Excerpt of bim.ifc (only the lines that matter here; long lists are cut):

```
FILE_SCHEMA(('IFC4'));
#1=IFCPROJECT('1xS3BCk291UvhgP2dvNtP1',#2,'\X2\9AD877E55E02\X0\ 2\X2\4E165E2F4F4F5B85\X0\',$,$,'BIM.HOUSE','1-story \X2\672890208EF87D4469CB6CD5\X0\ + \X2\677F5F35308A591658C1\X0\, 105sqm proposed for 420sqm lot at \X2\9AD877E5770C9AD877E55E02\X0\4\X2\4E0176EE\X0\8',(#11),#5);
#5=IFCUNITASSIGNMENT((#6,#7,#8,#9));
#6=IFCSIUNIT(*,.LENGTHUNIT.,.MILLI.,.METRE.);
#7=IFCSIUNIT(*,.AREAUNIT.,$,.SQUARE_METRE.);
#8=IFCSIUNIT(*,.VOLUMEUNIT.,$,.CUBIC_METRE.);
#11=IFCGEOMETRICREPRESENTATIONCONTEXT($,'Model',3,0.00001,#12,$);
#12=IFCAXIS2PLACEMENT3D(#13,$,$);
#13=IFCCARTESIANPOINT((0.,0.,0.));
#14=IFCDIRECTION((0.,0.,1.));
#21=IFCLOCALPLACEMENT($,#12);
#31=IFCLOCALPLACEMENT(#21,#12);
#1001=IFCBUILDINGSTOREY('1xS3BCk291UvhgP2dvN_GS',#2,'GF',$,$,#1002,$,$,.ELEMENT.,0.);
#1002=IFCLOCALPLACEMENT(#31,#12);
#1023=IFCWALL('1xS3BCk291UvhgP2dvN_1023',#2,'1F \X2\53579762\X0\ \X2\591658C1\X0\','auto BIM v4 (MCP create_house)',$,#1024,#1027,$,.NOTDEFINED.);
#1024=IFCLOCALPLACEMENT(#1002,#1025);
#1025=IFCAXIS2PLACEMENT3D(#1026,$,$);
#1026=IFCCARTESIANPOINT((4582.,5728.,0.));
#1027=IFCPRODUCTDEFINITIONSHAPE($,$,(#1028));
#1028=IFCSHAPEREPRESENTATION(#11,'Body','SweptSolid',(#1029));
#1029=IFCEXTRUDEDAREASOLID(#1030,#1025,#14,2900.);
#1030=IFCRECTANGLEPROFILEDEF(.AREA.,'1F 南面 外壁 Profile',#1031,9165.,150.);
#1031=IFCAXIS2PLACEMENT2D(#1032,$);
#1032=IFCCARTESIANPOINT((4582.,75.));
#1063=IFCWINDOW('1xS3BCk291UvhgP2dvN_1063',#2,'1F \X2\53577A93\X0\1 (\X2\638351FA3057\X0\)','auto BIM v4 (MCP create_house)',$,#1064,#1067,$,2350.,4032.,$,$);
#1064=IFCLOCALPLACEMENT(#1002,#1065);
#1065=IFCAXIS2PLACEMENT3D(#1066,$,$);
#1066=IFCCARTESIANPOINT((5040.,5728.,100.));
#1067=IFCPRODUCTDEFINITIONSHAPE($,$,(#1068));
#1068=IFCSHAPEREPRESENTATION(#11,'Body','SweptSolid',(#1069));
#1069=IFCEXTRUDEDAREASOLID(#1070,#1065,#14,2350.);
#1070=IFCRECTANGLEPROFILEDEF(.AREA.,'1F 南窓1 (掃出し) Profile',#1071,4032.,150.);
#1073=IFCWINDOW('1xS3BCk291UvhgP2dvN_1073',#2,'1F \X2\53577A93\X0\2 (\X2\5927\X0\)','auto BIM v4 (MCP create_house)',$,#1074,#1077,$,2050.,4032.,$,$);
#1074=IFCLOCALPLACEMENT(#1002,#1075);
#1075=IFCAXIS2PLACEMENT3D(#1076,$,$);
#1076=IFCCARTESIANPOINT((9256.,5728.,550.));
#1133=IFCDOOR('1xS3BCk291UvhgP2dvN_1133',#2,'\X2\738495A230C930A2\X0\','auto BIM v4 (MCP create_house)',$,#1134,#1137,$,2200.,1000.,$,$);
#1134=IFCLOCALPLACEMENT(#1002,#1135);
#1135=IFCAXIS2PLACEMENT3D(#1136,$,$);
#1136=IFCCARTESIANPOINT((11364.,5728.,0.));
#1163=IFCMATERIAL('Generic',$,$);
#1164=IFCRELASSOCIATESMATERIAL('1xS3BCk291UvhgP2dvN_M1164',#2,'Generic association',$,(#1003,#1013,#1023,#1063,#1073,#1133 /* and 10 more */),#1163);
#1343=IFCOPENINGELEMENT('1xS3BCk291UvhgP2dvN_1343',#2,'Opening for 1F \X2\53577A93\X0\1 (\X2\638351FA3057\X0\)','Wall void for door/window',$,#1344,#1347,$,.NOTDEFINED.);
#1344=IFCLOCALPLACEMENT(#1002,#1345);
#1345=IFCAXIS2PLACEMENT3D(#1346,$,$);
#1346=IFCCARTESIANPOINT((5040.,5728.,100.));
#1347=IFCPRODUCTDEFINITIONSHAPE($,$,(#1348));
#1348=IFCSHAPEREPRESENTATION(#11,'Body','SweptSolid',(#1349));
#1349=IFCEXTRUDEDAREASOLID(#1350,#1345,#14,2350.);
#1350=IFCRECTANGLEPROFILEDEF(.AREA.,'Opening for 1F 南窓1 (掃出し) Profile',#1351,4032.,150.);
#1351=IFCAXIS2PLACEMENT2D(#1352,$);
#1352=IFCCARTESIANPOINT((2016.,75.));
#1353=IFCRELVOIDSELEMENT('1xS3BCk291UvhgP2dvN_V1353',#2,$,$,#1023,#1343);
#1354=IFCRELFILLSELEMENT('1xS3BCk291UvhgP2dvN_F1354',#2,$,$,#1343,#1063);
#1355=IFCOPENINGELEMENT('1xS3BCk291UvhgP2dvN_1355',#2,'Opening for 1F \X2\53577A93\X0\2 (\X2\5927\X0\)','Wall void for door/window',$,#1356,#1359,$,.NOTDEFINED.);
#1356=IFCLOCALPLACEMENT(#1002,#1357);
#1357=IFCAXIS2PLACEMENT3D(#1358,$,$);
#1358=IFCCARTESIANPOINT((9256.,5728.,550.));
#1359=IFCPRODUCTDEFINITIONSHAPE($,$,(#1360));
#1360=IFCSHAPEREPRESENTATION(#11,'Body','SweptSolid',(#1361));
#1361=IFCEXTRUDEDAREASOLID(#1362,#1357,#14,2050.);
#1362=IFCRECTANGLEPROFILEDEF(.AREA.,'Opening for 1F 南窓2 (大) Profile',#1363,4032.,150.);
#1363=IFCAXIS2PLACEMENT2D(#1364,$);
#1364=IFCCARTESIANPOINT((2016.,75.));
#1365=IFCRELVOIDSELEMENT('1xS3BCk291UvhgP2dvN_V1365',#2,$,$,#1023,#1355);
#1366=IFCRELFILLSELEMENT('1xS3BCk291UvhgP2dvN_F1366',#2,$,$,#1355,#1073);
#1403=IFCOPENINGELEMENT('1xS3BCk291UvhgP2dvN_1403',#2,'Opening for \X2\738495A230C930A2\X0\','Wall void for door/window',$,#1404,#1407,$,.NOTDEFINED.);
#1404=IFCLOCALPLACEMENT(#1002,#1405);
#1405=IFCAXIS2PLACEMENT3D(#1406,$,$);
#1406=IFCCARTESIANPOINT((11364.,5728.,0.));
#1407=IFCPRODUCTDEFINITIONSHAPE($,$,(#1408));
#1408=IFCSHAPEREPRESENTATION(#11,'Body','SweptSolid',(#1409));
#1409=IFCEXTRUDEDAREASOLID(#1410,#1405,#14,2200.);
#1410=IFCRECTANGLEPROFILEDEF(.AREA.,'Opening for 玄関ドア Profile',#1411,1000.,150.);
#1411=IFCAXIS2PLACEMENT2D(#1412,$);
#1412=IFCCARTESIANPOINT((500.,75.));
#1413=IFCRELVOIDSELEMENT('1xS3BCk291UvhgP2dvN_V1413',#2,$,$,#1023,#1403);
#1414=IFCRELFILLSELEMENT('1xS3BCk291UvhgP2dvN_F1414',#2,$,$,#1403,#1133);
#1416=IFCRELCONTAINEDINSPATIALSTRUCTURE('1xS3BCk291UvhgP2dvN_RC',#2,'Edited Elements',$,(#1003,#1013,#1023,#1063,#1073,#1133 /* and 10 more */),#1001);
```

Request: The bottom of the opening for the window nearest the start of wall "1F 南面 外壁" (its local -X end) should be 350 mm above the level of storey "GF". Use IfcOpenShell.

```python
import numpy as np
import ifcopenshell
import ifcopenshell.api.geometry
import ifcopenshell.geom
import ifcopenshell.util.element
import ifcopenshell.util.placement
import ifcopenshell.util.shape
import ifcopenshell.util.unit

model = ifcopenshell.open("bim.ifc")
unit_scale = ifcopenshell.util.unit.calculate_unit_scale(model)

window = model.by_guid("1xS3BCk291UvhgP2dvN_1063")
opening = window.FillsVoids[0].RelatingOpeningElement
storey = ifcopenshell.util.element.get_container(window, ifc_class="IfcBuildingStorey")
level = ifcopenshell.util.placement.get_local_placement(storey.ObjectPlacement)[2, 3]

# The opening's origin need not be at the sill, so measure its lowest point.
shape = ifcopenshell.geom.create_shape(ifcopenshell.geom.settings(), opening)
bottom = ifcopenshell.util.shape.get_shape_bottom_elevation(shape, shape.geometry) / unit_scale
dz = level + 0.35 / unit_scale - bottom

shift = np.array([0.0, 0.0, dz])
# The window is not placed relative to its opening, so move both.
for product in (opening, window):
    matrix = ifcopenshell.util.placement.get_local_placement(product.ObjectPlacement)
    matrix[:3, 3] += shift
    ifcopenshell.api.geometry.edit_object_placement(model, product=product, matrix=matrix, is_si=False)

print(f"moved by {dz * unit_scale:+.3f} m")

model.write("bim_edited.ifc")
```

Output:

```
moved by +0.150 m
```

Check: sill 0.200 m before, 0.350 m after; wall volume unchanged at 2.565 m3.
